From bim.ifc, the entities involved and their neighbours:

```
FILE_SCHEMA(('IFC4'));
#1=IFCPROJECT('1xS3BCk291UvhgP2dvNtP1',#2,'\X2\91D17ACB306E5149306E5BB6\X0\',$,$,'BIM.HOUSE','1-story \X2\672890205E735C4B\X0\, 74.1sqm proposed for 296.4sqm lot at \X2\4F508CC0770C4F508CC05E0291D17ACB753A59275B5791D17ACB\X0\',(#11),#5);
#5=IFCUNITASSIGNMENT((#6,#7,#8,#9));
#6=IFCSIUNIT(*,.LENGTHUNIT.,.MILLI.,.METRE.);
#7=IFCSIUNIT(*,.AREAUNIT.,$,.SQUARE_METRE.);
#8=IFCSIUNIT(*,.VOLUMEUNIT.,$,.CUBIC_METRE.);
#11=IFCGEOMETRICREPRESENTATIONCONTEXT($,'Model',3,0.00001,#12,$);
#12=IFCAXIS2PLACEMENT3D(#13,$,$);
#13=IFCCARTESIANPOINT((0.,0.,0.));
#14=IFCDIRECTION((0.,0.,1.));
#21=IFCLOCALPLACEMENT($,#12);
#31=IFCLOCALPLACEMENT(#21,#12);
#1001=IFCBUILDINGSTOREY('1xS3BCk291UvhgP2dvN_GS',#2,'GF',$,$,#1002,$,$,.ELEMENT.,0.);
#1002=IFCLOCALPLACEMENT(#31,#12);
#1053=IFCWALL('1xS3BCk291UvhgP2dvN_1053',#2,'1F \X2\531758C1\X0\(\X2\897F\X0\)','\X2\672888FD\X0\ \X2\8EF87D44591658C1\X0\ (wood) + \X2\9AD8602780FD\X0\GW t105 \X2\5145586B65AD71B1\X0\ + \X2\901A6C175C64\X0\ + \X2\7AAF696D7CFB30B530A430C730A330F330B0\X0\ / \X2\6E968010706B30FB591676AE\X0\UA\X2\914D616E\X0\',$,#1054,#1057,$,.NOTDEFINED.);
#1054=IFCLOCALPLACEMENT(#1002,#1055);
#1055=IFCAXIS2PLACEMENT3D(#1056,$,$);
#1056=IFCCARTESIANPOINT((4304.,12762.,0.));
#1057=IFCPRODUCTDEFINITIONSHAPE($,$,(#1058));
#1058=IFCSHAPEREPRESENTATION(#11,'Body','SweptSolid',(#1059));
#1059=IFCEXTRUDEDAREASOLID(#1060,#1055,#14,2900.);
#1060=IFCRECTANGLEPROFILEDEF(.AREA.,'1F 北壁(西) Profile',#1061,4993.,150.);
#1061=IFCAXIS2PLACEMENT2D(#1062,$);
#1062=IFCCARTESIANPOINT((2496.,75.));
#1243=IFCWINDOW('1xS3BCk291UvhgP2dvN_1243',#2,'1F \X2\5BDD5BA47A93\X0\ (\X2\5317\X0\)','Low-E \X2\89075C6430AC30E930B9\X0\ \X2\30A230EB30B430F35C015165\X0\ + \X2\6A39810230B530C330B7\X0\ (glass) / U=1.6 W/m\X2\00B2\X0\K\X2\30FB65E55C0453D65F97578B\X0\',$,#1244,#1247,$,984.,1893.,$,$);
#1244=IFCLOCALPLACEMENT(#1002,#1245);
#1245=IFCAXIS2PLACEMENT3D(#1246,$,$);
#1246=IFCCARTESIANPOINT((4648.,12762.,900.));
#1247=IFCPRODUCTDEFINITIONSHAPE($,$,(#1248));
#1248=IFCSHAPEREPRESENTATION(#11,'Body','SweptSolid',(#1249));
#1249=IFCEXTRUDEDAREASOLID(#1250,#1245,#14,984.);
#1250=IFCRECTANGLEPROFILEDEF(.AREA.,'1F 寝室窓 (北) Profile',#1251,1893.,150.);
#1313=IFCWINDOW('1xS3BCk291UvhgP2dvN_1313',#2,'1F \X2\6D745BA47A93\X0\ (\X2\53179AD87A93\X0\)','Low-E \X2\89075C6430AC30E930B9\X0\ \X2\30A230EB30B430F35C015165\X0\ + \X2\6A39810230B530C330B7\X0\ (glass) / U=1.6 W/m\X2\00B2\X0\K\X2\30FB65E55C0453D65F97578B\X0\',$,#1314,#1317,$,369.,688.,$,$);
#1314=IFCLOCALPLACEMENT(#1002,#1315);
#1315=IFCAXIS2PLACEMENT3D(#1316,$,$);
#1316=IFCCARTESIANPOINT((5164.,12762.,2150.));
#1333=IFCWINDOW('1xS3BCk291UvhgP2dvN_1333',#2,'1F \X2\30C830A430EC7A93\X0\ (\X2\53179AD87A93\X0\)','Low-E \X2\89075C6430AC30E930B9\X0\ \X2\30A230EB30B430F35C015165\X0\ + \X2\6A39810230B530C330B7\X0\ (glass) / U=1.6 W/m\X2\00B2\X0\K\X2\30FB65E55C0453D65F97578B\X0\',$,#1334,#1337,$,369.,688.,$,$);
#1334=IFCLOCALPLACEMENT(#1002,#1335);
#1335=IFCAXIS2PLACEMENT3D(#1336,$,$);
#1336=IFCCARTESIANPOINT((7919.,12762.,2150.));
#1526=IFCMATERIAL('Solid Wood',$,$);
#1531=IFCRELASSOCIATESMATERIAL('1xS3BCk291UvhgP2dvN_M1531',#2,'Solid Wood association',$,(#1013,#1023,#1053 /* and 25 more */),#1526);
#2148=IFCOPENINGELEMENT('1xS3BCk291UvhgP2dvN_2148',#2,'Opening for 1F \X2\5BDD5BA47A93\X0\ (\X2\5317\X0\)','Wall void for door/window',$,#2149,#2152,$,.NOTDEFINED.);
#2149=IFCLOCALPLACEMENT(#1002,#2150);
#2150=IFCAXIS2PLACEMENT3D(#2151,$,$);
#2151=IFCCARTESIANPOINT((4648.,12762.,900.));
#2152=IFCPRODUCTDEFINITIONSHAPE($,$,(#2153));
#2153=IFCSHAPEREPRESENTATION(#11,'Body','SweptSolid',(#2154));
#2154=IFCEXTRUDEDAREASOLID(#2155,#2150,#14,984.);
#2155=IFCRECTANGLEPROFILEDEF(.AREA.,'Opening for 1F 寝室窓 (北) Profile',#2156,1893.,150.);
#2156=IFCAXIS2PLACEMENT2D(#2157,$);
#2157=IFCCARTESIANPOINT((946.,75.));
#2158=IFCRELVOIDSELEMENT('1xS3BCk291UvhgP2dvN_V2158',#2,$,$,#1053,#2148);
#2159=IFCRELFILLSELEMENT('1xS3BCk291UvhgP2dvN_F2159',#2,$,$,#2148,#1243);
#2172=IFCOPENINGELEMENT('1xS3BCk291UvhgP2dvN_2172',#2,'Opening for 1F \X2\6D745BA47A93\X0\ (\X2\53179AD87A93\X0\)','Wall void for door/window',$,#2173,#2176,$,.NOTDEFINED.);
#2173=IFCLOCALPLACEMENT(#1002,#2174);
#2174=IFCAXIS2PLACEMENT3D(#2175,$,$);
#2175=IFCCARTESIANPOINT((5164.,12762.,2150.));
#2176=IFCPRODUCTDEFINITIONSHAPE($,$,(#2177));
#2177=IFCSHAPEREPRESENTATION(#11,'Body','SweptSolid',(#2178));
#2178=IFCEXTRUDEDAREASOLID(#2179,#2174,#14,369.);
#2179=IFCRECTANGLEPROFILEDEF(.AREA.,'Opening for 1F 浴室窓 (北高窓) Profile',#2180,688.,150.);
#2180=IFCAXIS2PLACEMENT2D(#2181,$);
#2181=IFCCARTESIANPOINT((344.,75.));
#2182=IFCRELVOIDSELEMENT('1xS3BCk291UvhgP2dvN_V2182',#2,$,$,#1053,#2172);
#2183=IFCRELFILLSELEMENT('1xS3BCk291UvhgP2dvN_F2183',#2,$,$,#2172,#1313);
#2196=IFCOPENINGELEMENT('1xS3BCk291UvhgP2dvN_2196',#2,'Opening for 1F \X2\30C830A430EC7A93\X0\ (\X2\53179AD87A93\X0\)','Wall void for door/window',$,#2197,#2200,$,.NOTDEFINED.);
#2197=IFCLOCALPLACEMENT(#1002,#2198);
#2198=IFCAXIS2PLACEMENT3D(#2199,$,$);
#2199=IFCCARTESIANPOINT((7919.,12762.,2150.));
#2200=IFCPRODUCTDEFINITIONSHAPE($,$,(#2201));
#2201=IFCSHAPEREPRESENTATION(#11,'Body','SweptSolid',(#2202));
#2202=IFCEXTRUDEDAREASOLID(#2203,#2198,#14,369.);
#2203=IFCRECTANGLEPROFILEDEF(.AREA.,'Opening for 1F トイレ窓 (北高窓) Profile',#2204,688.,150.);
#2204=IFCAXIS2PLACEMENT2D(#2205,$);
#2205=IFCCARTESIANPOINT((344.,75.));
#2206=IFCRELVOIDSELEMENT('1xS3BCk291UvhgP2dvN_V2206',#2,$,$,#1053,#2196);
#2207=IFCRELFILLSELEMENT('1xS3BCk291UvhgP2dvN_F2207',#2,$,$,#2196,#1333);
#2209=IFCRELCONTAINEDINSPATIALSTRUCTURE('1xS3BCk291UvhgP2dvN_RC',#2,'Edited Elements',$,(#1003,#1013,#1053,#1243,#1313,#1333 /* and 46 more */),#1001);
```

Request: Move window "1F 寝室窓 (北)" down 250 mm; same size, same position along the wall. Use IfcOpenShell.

```python
import numpy as np
import ifcopenshell
import ifcopenshell.api.geometry
import ifcopenshell.util.placement
import ifcopenshell.util.unit

model = ifcopenshell.open("bim.ifc")
unit_scale = ifcopenshell.util.unit.calculate_unit_scale(model)

window = model.by_id(1243)
opening = window.FillsVoids[0].RelatingOpeningElement
dz = -0.25 / unit_scale

shift = np.array([0.0, 0.0, dz])
# The window is not placed relative to its opening, so move both.
for product in (opening, window):
    matrix = ifcopenshell.util.placement.get_local_placement(product.ObjectPlacement)
    matrix[:3, 3] += shift
    ifcopenshell.api.geometry.edit_object_placement(model, product=product, matrix=matrix, is_si=False)

print(f"moved by {dz * unit_scale:+.3f} m")

model.write("bim_updated.ifc")
```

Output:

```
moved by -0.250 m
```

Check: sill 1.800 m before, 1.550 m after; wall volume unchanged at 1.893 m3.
